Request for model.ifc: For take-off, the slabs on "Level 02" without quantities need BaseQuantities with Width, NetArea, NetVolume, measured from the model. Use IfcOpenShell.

First a look at what the model holds.

```python
import ifcopenshell
import ifcopenshell.util.element
import ifcopenshell.util.unit

model = ifcopenshell.open("model.ifc")
print(model.schema)
for unit_type in ("LENGTHUNIT", "AREAUNIT", "VOLUMEUNIT"):
    print(unit_type, ifcopenshell.util.unit.calculate_unit_scale(model, unit_type))
storey = next(s for s in model.by_type("IfcBuildingStorey") if s.Name == "Level 02")
slabs = [e for e in ifcopenshell.util.element.get_decomposition(storey) if e.is_a("IfcSlab")]
for e in sorted(slabs, key=lambda e: e.id()):
    print(e.id(), e.is_a(), e.Name, list(ifcopenshell.util.element.get_psets(e, qtos_only=True)), sep=" | ")
```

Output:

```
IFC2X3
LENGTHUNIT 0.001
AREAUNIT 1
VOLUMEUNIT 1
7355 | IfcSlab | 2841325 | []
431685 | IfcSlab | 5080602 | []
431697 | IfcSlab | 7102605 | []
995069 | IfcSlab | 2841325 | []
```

```python
import ifcopenshell
import ifcopenshell.api.pset
import ifcopenshell.geom
import ifcopenshell.util.element
import ifcopenshell.util.shape
import ifcopenshell.util.unit

model = ifcopenshell.open("model.ifc")
unit_scale = ifcopenshell.util.unit.calculate_unit_scale(model)
area_scale = ifcopenshell.util.unit.calculate_unit_scale(model, "AREAUNIT")
volume_scale = ifcopenshell.util.unit.calculate_unit_scale(model, "VOLUMEUNIT")
settings = ifcopenshell.geom.settings()

storey = next(s for s in model.by_type("IfcBuildingStorey") if s.Name == "Level 02")
slabs = [e for e in ifcopenshell.util.element.get_decomposition(storey) if e.is_a("IfcSlab")]

for e in sorted(slabs, key=lambda e: e.id()):
    if ifcopenshell.util.element.get_psets(e, qtos_only=True, should_inherit=False):
        continue
    # Geometry comes back in metres, in the element's own axes.
    shape = ifcopenshell.geom.create_shape(settings, e)
    values = {
        "Width": ifcopenshell.util.shape.get_z(shape.geometry) / unit_scale,
        "NetArea": ifcopenshell.util.shape.get_footprint_area(shape.geometry) / area_scale,
        "NetVolume": ifcopenshell.util.shape.get_volume(shape.geometry) / volume_scale,
    }
    qto = ifcopenshell.api.pset.add_qto(model, product=e, name="BaseQuantities")
    ifcopenshell.api.pset.edit_qto(model, qto=qto, properties=values)
    print(e.id(), {k: round(v, 3) for k, v in values.items()})

model.write("model_edited.ifc")
```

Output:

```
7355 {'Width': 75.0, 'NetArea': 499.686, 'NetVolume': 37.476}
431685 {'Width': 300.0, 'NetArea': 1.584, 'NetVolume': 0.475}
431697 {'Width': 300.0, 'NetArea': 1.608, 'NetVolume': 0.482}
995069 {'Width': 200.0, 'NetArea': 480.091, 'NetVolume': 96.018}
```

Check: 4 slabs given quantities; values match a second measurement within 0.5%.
